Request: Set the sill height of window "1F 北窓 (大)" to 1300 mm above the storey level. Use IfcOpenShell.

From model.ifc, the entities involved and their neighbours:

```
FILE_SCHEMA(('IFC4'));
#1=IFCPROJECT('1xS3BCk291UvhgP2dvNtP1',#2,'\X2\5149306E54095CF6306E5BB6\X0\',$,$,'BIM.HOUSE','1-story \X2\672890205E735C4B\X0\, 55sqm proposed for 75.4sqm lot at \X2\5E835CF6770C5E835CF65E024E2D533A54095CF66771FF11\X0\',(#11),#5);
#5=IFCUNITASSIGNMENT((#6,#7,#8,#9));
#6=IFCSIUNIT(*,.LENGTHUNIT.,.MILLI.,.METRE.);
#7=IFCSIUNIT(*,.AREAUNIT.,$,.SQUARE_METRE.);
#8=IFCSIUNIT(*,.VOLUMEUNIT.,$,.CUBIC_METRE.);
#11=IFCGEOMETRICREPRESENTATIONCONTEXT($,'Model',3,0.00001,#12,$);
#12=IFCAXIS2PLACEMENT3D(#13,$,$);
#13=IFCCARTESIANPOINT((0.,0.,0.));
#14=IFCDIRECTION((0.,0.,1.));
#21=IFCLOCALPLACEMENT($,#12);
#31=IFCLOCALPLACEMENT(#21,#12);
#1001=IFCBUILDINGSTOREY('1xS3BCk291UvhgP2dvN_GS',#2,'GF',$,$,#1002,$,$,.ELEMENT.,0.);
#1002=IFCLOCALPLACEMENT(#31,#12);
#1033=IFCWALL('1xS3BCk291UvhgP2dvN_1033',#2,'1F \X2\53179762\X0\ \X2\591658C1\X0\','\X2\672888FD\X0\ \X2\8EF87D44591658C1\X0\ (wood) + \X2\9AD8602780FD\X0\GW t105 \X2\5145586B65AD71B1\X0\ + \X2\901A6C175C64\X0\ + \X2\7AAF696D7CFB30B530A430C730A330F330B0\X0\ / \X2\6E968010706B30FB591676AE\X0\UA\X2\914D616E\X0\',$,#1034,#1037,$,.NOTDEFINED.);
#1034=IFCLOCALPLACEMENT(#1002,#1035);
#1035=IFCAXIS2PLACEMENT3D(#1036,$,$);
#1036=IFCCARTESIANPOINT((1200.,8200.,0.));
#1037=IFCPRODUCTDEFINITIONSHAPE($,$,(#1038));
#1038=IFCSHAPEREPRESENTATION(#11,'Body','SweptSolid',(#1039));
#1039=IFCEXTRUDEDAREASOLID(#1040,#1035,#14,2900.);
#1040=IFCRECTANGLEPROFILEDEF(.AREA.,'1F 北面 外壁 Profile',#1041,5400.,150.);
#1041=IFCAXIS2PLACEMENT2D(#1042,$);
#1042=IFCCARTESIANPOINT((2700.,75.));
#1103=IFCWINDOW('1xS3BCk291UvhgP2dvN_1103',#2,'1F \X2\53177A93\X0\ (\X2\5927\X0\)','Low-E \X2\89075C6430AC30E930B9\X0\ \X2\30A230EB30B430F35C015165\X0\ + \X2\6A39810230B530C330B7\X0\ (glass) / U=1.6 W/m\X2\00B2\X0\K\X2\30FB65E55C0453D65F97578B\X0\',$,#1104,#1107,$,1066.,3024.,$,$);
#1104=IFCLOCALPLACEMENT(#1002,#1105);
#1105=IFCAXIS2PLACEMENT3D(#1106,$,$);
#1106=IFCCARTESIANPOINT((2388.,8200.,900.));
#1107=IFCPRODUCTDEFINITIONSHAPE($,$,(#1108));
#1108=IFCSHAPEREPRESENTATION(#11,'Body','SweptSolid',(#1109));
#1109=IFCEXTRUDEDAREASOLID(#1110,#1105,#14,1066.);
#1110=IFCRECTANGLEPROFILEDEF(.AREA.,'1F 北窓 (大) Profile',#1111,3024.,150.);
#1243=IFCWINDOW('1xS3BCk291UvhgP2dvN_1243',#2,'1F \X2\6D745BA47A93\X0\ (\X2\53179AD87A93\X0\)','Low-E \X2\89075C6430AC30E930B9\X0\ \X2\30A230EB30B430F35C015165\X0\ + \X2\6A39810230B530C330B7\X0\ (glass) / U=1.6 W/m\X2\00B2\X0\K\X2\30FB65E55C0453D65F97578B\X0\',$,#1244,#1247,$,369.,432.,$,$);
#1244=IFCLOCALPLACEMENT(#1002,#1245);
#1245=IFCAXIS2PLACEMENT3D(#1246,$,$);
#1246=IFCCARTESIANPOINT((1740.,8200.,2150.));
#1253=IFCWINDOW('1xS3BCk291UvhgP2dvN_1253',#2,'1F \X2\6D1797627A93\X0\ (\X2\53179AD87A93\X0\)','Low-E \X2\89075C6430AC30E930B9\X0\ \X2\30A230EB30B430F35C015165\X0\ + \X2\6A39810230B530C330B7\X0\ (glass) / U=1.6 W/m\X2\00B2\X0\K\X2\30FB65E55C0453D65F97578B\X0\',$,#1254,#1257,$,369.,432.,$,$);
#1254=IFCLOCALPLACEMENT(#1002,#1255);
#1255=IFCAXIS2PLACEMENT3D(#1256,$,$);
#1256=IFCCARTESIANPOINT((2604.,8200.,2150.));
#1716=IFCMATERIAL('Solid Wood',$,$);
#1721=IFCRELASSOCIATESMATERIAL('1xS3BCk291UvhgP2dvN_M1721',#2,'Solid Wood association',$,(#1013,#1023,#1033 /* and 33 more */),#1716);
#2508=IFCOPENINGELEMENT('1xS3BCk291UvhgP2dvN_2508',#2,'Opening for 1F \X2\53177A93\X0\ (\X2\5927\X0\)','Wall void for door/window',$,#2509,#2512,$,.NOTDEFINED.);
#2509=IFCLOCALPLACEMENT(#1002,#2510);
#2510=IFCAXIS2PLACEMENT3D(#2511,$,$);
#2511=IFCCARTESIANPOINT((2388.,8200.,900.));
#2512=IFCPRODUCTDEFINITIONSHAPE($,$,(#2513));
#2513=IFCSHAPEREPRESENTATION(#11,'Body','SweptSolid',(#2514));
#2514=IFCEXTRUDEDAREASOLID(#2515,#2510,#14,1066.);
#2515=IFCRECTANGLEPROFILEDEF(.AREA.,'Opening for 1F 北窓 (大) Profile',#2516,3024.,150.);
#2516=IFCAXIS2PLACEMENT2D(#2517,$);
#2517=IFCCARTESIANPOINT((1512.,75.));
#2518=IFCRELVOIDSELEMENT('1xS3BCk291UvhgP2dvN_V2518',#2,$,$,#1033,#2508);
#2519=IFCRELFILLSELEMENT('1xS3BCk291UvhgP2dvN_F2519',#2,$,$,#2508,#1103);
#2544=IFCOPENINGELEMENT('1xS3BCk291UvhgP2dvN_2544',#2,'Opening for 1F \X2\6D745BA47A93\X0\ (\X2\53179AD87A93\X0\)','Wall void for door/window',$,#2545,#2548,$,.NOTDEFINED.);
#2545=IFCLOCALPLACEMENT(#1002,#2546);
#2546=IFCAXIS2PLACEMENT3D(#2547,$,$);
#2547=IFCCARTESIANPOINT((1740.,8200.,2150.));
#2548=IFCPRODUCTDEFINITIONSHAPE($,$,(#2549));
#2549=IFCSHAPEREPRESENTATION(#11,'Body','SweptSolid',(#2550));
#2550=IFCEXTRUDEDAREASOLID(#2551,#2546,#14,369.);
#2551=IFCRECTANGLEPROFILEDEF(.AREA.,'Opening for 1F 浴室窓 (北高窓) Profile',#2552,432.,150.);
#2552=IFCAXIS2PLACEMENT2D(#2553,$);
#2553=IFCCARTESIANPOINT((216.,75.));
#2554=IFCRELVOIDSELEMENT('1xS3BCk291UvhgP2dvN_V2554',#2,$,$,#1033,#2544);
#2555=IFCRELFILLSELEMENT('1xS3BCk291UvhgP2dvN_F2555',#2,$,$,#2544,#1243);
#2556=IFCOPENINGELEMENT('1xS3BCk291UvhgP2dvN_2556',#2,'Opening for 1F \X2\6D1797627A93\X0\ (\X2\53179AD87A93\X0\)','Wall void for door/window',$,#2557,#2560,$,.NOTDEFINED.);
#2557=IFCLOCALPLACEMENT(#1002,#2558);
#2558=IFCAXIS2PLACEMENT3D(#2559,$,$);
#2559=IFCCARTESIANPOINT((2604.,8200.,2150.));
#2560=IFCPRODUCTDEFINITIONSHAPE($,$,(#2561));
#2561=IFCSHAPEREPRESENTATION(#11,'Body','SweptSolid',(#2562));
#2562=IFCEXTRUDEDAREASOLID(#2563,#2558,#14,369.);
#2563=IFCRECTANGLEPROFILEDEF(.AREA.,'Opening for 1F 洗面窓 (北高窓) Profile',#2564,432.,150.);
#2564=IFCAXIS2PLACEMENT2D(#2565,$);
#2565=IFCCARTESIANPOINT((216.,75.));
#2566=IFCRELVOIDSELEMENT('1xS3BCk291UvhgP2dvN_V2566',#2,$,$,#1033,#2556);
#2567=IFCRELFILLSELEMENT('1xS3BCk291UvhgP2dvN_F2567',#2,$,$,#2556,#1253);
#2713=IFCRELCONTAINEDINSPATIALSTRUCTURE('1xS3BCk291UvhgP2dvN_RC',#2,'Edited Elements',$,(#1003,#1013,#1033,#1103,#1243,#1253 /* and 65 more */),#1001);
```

```python
import numpy as np
import ifcopenshell
import ifcopenshell.api.geometry
import ifcopenshell.geom
import ifcopenshell.util.element
import ifcopenshell.util.placement
import ifcopenshell.util.shape
import ifcopenshell.util.unit

model = ifcopenshell.open("model.ifc")
unit_scale = ifcopenshell.util.unit.calculate_unit_scale(model)

window = model.by_id(1103)
opening = window.FillsVoids[0].RelatingOpeningElement
storey = ifcopenshell.util.element.get_container(window, ifc_class="IfcBuildingStorey")
level = ifcopenshell.util.placement.get_local_placement(storey.ObjectPlacement)[2, 3]

# The opening's origin need not be at the sill, so measure its lowest point.
shape = ifcopenshell.geom.create_shape(ifcopenshell.geom.settings(), opening)
bottom = ifcopenshell.util.shape.get_shape_bottom_elevation(shape, shape.geometry) / unit_scale
dz = level + 1300.0 - bottom

shift = np.array([0.0, 0.0, dz])
# The window is not placed relative to its opening, so move both.
for product in (opening, window):
    matrix = ifcopenshell.util.placement.get_local_placement(product.ObjectPlacement)
    matrix[:3, 3] += shift
    ifcopenshell.api.geometry.edit_object_placement(model, product=product, matrix=matrix, is_si=False)

print(f"moved by {dz * unit_scale:+.3f} m")

model.write("model-out.ifc")
```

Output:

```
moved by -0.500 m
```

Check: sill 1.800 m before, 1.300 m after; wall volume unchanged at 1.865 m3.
